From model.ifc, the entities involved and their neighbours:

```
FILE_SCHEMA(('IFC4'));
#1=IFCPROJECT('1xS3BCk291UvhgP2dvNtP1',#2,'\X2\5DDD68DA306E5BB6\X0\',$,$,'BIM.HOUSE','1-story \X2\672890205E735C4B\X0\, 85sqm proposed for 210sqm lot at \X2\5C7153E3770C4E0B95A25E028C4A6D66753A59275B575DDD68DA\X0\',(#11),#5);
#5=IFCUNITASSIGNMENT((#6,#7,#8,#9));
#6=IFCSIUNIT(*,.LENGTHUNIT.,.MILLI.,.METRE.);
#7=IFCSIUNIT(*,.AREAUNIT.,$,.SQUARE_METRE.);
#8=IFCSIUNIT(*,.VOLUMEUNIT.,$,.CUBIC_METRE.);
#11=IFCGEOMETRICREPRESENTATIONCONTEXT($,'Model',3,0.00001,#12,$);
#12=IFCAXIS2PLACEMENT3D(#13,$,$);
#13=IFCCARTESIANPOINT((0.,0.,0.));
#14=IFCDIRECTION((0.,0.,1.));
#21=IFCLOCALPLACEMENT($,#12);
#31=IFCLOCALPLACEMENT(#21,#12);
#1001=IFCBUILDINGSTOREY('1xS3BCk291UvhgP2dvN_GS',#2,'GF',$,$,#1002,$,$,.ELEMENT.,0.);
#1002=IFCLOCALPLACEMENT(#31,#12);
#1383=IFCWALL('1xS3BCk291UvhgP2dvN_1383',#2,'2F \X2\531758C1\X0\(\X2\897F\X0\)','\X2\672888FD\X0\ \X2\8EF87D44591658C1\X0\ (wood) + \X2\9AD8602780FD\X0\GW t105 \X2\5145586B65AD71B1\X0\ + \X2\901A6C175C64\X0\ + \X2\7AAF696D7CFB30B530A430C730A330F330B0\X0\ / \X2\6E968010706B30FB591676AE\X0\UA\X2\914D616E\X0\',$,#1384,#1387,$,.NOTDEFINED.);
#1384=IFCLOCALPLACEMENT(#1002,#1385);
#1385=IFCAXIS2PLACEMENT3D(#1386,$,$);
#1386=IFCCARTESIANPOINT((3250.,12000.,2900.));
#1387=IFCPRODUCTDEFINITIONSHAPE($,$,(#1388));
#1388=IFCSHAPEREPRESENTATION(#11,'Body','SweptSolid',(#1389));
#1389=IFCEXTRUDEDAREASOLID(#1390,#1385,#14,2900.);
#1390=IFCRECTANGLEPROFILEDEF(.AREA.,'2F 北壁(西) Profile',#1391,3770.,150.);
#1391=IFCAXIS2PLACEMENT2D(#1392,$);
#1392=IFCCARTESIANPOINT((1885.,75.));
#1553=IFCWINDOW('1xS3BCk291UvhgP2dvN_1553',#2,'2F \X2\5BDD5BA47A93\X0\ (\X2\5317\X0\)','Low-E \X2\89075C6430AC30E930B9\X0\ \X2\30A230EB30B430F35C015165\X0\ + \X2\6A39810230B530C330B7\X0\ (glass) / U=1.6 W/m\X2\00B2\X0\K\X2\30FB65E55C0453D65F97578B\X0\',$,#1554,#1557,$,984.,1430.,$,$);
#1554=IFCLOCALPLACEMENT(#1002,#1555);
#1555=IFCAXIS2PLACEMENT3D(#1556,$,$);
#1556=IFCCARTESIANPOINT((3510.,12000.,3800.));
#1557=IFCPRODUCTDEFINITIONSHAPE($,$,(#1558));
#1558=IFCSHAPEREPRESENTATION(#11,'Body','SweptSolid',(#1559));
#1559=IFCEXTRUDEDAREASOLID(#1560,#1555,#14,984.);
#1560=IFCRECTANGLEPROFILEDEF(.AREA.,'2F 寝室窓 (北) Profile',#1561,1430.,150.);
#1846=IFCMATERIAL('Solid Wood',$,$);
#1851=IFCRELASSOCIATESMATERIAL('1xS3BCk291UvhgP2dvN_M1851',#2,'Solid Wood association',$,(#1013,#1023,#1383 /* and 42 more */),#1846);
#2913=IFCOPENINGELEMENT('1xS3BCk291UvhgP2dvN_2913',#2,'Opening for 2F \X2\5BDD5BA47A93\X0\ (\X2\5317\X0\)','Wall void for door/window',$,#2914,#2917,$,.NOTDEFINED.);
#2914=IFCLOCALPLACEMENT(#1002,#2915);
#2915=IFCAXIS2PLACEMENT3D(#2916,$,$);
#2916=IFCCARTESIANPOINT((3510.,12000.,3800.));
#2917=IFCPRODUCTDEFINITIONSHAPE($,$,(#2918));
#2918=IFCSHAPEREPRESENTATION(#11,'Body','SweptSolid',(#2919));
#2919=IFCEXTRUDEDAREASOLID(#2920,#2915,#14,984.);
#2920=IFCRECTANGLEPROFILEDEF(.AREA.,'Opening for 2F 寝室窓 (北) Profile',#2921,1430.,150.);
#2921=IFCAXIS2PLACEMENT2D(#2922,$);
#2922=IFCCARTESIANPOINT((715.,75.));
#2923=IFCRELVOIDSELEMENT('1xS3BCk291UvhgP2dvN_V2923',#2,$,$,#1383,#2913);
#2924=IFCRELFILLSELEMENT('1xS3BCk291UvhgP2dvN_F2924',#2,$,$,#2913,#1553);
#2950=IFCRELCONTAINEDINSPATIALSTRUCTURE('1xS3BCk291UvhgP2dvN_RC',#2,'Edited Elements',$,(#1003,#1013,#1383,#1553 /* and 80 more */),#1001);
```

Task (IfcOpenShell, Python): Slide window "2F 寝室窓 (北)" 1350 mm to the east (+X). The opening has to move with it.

```python
import ifcopenshell
import ifcopenshell.api.geometry
import ifcopenshell.util.placement
import ifcopenshell.util.unit

model = ifcopenshell.open("model.ifc")
unit_scale = ifcopenshell.util.unit.calculate_unit_scale(model)

window = model.by_guid("1xS3BCk291UvhgP2dvN_1553")
opening = window.FillsVoids[0].RelatingOpeningElement
wall = opening.VoidsElements[0].RelatingBuildingElement

wall_matrix = ifcopenshell.util.placement.get_local_placement(wall.ObjectPlacement)
shift = wall_matrix[:3, 0] * 1.35 / unit_scale
before = ifcopenshell.util.placement.get_local_placement(window.ObjectPlacement)[:3, 3].copy()

# The window is not placed relative to its opening, so move both.
for product in (opening, window):
    matrix = ifcopenshell.util.placement.get_local_placement(product.ObjectPlacement)
    matrix[:3, 3] += shift
    ifcopenshell.api.geometry.edit_object_placement(model, product=product, matrix=matrix, is_si=False)

after = ifcopenshell.util.placement.get_local_placement(window.ObjectPlacement)[:3, 3]
print("window moved by", (after - before).round(3) + 0.0)

model.write("model_updated.ifc")
```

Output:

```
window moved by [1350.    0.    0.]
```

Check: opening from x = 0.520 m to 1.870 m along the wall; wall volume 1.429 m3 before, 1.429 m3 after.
